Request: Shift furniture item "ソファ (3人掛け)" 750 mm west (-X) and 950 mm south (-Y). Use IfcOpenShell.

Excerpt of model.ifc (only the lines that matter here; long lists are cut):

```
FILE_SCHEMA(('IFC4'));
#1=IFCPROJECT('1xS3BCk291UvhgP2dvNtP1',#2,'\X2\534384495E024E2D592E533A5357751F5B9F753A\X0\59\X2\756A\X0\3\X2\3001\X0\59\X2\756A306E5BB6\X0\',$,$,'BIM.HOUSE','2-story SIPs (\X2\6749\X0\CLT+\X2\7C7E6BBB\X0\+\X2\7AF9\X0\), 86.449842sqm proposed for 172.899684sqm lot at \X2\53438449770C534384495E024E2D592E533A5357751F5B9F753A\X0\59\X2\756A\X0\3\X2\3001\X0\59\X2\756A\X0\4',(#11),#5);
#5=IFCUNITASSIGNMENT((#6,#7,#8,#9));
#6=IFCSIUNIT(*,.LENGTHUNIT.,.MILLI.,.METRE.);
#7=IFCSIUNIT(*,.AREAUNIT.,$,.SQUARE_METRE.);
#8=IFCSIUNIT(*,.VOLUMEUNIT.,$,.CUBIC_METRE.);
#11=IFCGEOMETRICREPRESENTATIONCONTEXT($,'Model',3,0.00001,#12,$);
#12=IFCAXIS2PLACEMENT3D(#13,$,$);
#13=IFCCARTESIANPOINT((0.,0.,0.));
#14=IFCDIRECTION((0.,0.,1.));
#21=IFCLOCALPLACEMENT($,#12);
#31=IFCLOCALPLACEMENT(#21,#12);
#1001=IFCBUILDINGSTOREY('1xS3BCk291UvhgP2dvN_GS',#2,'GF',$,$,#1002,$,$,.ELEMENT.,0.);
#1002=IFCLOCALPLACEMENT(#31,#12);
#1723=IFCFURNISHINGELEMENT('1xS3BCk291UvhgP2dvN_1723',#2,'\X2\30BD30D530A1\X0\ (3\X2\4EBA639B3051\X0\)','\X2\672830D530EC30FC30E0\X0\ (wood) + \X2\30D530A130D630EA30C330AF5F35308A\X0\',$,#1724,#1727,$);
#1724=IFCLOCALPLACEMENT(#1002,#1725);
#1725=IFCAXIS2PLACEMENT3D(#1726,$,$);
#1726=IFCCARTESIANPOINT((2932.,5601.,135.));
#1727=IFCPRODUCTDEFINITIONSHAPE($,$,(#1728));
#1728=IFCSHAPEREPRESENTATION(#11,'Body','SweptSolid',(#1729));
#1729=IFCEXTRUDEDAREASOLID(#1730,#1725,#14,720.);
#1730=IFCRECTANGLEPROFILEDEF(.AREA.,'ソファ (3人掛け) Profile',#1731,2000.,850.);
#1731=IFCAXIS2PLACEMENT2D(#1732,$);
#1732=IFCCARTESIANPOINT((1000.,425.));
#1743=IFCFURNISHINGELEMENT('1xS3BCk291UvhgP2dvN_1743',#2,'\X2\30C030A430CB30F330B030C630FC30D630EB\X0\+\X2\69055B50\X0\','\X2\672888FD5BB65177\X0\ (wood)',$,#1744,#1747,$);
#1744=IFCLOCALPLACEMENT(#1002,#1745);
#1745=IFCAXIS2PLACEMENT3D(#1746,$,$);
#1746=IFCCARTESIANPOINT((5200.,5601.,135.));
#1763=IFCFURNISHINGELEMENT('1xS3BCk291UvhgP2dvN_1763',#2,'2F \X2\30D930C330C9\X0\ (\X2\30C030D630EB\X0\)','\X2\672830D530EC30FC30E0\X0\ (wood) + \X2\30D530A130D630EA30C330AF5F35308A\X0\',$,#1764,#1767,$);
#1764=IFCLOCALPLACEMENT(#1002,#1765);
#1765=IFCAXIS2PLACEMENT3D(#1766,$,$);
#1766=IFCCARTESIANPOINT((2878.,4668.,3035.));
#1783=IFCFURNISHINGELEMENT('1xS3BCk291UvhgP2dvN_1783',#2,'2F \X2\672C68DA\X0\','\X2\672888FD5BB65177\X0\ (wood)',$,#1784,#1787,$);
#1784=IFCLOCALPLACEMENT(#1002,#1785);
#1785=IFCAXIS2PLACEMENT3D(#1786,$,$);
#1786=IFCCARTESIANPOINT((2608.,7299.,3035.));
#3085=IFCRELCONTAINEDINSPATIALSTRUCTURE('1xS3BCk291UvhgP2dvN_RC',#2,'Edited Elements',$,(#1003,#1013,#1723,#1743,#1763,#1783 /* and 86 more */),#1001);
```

```python
import ifcopenshell
import ifcopenshell.api.geometry
import ifcopenshell.util.placement

model = ifcopenshell.open("model.ifc")

item = model.by_id(1723)
matrix = ifcopenshell.util.placement.get_local_placement(item.ObjectPlacement)
matrix[0, 3] -= 750.0
matrix[1, 3] -= 950.0
ifcopenshell.api.geometry.edit_object_placement(model, product=item, matrix=matrix, is_si=False)

print(ifcopenshell.util.placement.get_local_placement(item.ObjectPlacement).round(3) + 0.0)

model.write("model_rev.ifc")
```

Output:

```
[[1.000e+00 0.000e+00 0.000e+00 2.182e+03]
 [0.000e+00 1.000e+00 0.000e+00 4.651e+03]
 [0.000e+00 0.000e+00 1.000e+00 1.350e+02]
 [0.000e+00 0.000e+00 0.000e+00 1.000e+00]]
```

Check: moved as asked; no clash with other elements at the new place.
